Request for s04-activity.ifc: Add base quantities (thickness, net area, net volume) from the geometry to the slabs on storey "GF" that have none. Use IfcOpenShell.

First a look at what the model holds.

```python
import ifcopenshell
import ifcopenshell.util.element
import ifcopenshell.util.unit

model = ifcopenshell.open("s04-activity.ifc")
print(model.schema)
for unit_type in ("LENGTHUNIT", "AREAUNIT", "VOLUMEUNIT"):
    print(unit_type, ifcopenshell.util.unit.calculate_unit_scale(model, unit_type))
storey = next(s for s in model.by_type("IfcBuildingStorey") if s.Name == "GF")
slabs = [e for e in ifcopenshell.util.element.get_decomposition(storey) if e.is_a("IfcSlab")]
for e in sorted(slabs, key=lambda e: e.id()):
    print(e.id(), e.is_a(), e.Name, list(ifcopenshell.util.element.get_psets(e, qtos_only=True)), sep=" | ")
```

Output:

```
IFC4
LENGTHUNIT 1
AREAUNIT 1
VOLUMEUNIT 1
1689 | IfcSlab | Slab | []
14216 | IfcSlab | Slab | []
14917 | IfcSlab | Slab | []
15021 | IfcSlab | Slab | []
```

```python
import ifcopenshell
import ifcopenshell.api.pset
import ifcopenshell.geom
import ifcopenshell.util.element
import ifcopenshell.util.shape
import ifcopenshell.util.unit

model = ifcopenshell.open("s04-activity.ifc")
unit_scale = ifcopenshell.util.unit.calculate_unit_scale(model)
area_scale = ifcopenshell.util.unit.calculate_unit_scale(model, "AREAUNIT")
volume_scale = ifcopenshell.util.unit.calculate_unit_scale(model, "VOLUMEUNIT")
settings = ifcopenshell.geom.settings()

storey = next(s for s in model.by_type("IfcBuildingStorey") if s.Name == "GF")
slabs = [e for e in ifcopenshell.util.element.get_decomposition(storey) if e.is_a("IfcSlab")]

for e in sorted(slabs, key=lambda e: e.id()):
    if ifcopenshell.util.element.get_psets(e, qtos_only=True, should_inherit=False):
        continue
    # Geometry comes back in metres, in the element's own axes.
    shape = ifcopenshell.geom.create_shape(settings, e)
    values = {
        "Width": ifcopenshell.util.shape.get_z(shape.geometry) / unit_scale,
        "NetArea": ifcopenshell.util.shape.get_footprint_area(shape.geometry) / area_scale,
        "NetVolume": ifcopenshell.util.shape.get_volume(shape.geometry) / volume_scale,
    }
    qto = ifcopenshell.api.pset.add_qto(model, product=e, name="Qto_SlabBaseQuantities")
    ifcopenshell.api.pset.edit_qto(model, qto=qto, properties=values)
    print(e.id(), {k: round(v, 3) for k, v in values.items()})

model.write("s04-activity_updated.ifc")
```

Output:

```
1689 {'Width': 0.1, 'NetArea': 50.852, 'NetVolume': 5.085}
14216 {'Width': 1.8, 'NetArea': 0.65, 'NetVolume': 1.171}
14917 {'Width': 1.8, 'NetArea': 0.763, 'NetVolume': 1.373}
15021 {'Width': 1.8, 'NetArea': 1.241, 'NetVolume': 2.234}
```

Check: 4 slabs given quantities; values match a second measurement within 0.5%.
